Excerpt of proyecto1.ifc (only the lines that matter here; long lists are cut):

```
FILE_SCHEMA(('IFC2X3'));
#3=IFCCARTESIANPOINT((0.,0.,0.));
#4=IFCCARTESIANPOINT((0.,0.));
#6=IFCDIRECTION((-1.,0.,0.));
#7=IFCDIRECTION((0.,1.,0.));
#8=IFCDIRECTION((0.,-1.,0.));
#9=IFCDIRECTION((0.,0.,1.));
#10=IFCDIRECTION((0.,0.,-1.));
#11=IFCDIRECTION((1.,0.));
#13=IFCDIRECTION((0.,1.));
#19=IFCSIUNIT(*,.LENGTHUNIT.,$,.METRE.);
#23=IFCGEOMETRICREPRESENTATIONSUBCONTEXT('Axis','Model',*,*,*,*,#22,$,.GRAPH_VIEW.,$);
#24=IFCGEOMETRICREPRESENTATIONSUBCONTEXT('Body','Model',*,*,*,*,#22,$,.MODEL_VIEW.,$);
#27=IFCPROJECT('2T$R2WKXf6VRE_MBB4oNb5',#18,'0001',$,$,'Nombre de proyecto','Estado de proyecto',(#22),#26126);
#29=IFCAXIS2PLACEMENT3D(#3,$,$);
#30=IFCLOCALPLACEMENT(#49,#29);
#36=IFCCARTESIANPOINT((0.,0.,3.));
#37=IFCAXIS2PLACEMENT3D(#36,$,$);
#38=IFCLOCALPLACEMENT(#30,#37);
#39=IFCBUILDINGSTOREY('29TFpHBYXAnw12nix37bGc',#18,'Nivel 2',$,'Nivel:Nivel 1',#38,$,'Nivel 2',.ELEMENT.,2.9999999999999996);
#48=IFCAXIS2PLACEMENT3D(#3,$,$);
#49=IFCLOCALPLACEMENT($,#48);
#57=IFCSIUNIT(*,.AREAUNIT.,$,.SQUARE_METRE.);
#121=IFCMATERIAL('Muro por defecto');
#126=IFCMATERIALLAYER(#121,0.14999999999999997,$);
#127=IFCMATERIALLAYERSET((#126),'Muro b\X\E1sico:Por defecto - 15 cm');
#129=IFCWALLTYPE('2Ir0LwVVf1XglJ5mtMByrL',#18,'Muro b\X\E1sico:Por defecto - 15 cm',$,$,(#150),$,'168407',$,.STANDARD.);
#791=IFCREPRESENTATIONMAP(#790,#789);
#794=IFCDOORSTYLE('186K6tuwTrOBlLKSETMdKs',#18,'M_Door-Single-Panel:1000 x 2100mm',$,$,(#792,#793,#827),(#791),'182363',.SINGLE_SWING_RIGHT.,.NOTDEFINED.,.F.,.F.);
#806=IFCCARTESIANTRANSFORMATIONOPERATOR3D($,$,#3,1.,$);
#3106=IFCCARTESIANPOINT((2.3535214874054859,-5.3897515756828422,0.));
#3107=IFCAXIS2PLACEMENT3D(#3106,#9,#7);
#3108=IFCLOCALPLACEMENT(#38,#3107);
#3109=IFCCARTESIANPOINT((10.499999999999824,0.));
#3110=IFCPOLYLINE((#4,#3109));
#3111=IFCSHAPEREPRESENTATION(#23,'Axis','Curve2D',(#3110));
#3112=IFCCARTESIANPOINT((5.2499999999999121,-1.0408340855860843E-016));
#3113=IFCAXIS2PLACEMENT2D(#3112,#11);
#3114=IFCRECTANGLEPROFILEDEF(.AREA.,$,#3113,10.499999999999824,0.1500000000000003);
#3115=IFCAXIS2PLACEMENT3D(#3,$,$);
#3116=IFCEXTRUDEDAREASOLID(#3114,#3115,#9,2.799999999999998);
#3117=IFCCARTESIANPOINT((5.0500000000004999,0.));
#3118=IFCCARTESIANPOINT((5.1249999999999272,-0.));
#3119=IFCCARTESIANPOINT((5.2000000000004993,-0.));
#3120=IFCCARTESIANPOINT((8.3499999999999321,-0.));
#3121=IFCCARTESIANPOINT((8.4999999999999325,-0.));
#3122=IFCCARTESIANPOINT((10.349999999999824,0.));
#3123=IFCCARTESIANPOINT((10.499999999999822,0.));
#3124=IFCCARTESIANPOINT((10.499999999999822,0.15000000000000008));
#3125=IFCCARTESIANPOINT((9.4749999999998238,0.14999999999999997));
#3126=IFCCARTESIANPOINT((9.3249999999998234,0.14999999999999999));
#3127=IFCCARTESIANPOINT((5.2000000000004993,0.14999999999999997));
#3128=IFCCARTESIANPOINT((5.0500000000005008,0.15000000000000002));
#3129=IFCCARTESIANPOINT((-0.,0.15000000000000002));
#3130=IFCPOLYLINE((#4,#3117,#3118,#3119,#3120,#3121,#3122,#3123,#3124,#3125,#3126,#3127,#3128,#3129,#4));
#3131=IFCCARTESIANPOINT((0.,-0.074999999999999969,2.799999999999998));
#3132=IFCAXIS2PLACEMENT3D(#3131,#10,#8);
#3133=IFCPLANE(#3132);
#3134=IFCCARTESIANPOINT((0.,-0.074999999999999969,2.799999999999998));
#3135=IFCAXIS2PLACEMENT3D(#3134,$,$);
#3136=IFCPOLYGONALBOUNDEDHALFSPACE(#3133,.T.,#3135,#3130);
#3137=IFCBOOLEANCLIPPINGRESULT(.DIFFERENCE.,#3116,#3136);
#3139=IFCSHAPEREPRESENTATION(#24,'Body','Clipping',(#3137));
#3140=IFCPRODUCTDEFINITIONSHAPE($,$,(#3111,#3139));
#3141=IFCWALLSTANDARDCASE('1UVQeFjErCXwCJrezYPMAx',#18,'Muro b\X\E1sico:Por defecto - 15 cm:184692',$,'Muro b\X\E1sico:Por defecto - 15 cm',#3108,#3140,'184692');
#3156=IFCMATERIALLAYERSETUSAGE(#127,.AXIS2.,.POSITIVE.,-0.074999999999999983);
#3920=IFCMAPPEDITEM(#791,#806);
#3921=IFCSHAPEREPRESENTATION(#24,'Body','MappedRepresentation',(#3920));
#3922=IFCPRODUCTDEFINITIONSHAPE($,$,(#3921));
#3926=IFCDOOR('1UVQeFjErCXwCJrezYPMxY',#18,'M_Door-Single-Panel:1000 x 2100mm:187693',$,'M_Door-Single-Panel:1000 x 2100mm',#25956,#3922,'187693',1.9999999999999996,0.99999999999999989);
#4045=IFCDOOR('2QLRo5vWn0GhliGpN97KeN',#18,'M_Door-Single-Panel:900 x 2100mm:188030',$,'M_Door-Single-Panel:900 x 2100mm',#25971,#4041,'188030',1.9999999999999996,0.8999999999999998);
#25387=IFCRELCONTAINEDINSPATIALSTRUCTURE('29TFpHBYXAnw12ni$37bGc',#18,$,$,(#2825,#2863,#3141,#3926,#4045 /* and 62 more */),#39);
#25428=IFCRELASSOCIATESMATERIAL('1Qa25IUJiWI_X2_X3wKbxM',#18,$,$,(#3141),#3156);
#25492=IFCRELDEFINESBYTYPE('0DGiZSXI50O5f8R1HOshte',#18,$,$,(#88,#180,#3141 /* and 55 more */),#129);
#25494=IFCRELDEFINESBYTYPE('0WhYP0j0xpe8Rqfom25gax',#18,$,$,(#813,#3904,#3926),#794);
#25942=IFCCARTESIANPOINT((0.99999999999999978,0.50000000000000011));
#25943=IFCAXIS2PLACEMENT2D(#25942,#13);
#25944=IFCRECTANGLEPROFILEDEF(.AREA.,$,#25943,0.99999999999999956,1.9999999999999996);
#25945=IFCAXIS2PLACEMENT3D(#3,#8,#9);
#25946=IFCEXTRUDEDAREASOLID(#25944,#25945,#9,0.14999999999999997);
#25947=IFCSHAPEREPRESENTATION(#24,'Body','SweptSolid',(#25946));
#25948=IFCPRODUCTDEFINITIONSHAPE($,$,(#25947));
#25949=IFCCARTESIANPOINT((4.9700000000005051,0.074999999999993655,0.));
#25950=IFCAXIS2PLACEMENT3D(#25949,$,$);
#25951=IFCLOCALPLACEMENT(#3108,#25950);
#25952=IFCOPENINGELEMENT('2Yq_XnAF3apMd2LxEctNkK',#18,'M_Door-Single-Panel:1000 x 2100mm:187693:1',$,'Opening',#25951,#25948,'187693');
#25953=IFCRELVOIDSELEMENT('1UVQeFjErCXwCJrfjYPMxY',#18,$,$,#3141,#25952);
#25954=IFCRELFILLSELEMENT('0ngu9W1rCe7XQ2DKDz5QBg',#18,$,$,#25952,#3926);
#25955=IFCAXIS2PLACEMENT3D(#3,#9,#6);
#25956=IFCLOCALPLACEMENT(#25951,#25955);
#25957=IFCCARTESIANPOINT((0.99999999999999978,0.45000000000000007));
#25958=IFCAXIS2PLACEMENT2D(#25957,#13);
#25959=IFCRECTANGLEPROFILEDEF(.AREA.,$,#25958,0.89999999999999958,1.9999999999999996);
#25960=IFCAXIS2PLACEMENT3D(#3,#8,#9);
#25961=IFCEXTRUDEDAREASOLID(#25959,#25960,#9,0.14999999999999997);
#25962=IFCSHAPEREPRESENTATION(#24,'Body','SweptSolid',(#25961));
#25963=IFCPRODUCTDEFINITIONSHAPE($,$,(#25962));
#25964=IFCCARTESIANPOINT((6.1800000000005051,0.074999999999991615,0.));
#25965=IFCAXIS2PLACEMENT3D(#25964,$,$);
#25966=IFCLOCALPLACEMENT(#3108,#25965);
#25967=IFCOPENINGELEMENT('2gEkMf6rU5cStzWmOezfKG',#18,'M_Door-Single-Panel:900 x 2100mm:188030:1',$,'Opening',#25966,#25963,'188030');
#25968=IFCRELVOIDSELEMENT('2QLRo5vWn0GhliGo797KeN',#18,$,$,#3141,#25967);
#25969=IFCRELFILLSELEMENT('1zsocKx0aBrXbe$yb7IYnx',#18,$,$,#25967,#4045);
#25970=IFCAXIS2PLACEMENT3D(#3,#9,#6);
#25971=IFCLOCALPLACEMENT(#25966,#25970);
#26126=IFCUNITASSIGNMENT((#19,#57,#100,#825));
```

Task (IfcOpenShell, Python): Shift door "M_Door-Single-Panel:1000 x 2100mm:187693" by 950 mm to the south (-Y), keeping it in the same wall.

```python
import ifcopenshell
import ifcopenshell.api.geometry
import ifcopenshell.util.placement
import ifcopenshell.util.unit

model = ifcopenshell.open("proyecto1.ifc")
unit_scale = ifcopenshell.util.unit.calculate_unit_scale(model)

door = model.by_guid("1UVQeFjErCXwCJrezYPMxY")
opening = door.FillsVoids[0].RelatingOpeningElement
wall = opening.VoidsElements[0].RelatingBuildingElement

wall_matrix = ifcopenshell.util.placement.get_local_placement(wall.ObjectPlacement)
shift = wall_matrix[:3, 0] * -0.95 / unit_scale
before = ifcopenshell.util.placement.get_local_placement(door.ObjectPlacement)[:3, 3].copy()

# The door is placed relative to its opening, so it follows when the opening moves.
matrix = ifcopenshell.util.placement.get_local_placement(opening.ObjectPlacement)
matrix[:3, 3] += shift
ifcopenshell.api.geometry.edit_object_placement(
    model, product=opening, matrix=matrix, is_si=False, should_transform_children=True
)

after = ifcopenshell.util.placement.get_local_placement(door.ObjectPlacement)[:3, 3]
print("door moved by", (after - before).round(3) + 0.0)

model.write("proyecto1_rev.ifc")
```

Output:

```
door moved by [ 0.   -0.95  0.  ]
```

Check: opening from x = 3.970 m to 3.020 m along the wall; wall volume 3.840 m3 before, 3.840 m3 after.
